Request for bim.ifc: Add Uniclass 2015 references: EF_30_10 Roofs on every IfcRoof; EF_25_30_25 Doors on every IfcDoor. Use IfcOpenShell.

First a look at what the model holds.

```python
import ifcopenshell

model = ifcopenshell.open("bim.ifc")
print(model.schema)
print("classifications:", [c.Name for c in model.by_type("IfcClassification")])
for ifc_class in ("IfcDoor", "IfcRoof", "IfcStair", "IfcWall", "IfcWindow"):
    print(ifc_class, len(model.by_type(ifc_class)))
```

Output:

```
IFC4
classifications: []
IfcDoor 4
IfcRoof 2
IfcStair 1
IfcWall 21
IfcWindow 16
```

```python
import ifcopenshell
import ifcopenshell.api.classification

model = ifcopenshell.open("bim.ifc")

system = ifcopenshell.api.classification.add_classification(model, classification="Uniclass 2015")

codes = {
    "IfcRoof": ("EF_30_10", "Roofs"),
    "IfcDoor": ("EF_25_30_25", "Doors"),
}
for ifc_class, (code, name) in codes.items():
    products = model.by_type(ifc_class)
    ifcopenshell.api.classification.add_reference(
        model, products=products, classification=system, identification=code, name=name
    )
    print(code, len(products))

model.write("bim_v2.ifc")
```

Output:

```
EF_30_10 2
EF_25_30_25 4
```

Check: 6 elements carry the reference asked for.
